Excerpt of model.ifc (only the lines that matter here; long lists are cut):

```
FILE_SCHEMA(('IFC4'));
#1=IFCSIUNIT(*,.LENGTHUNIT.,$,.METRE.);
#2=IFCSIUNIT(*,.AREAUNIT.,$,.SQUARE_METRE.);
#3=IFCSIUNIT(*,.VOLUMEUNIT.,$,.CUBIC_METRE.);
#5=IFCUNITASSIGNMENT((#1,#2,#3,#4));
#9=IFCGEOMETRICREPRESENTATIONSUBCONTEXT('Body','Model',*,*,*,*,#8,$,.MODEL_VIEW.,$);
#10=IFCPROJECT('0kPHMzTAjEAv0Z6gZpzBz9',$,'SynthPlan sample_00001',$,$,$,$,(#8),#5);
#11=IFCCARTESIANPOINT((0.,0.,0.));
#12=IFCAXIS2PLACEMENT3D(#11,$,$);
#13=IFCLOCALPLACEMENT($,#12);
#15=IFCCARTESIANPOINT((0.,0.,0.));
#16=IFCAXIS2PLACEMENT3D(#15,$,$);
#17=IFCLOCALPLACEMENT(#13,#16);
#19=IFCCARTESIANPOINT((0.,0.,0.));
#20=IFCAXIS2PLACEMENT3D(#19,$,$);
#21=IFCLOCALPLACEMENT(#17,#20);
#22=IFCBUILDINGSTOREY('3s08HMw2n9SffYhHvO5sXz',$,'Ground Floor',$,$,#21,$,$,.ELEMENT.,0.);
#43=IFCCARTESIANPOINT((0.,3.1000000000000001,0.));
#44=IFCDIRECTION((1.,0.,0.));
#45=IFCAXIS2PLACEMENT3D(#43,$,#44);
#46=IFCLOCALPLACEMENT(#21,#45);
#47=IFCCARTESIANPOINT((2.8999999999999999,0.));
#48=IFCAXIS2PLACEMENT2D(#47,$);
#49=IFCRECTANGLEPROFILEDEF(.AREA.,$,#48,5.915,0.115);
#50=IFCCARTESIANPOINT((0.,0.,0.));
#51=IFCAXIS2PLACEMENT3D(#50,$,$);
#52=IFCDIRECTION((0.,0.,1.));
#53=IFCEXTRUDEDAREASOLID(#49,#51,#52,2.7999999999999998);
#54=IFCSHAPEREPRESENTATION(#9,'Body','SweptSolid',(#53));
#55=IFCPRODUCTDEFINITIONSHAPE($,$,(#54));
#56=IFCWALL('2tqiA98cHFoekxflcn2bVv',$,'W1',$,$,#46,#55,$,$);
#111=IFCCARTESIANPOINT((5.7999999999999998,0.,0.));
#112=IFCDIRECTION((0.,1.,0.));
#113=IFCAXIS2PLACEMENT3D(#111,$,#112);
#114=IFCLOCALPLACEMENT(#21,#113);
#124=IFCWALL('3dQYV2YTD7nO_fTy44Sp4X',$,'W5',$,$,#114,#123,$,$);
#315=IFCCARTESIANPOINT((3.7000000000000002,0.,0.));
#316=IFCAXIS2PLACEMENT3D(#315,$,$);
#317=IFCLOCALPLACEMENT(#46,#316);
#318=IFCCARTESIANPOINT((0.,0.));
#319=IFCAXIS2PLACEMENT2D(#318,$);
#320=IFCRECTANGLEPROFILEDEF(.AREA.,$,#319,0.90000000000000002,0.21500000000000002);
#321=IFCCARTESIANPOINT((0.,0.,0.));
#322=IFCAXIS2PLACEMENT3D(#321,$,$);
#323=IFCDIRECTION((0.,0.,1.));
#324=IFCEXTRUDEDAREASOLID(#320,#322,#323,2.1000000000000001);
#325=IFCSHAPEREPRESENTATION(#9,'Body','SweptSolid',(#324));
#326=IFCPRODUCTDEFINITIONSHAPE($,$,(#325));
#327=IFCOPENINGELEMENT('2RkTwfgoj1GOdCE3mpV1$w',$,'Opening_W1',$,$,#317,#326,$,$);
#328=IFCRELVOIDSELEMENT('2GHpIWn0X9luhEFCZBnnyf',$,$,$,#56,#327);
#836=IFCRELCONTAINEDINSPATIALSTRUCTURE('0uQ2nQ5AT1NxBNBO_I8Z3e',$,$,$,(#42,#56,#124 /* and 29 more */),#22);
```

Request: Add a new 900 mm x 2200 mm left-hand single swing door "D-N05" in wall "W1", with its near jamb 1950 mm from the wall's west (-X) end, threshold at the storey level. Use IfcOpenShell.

```python
import numpy as np
import ifcopenshell
import ifcopenshell.api.feature
import ifcopenshell.api.geometry
import ifcopenshell.api.root
import ifcopenshell.api.spatial
import ifcopenshell.geom
import ifcopenshell.util.element
import ifcopenshell.util.placement
import ifcopenshell.util.representation
import ifcopenshell.util.shape
import ifcopenshell.util.unit

model = ifcopenshell.open("model.ifc")
unit_scale = ifcopenshell.util.unit.calculate_unit_scale(model)
settings = ifcopenshell.geom.settings()


def volume(element):
    """Net volume in cubic metres, openings subtracted."""
    shape = ifcopenshell.geom.create_shape(settings, element)
    return ifcopenshell.util.shape.get_volume(shape.geometry)


wall = model.by_guid("2tqiA98cHFoekxflcn2bVv")
storey = ifcopenshell.util.element.get_container(wall, ifc_class="IfcBuildingStorey")
context = ifcopenshell.util.representation.get_context(model, "Model", "Body", "MODEL_VIEW")
before = volume(wall)

width, height, from_end, sill = 0.9, 2.2, 1.95, 0.0  # metres

# The wall runs along its own X axis, and the end named is its -X end.
wall_shape = ifcopenshell.geom.create_shape(settings, wall)
x, y, z = ifcopenshell.util.shape.get_vertices(wall_shape.geometry).T
start = x.min() + from_end
face, thickness = float(y.min()), float(y.max() - y.min())
wall_matrix = ifcopenshell.util.placement.get_local_placement(wall.ObjectPlacement)
level = ifcopenshell.util.placement.get_local_placement(storey.ObjectPlacement)[2, 3]


def in_wall(x, y):
    """Placement at x, y metres in the wall's axes, at sill height."""
    matrix = wall_matrix.copy()
    matrix[:, 3] = wall_matrix @ np.array([x / unit_scale, y / unit_scale, 0.0, 1.0])
    matrix[2, 3] = level + sill / unit_scale
    return matrix


# Opening: a box that overshoots both wall faces by 50 mm.
opening = ifcopenshell.api.root.create_entity(model, ifc_class="IfcOpeningElement", predefined_type="OPENING")
box = ifcopenshell.api.geometry.add_wall_representation(
    model, context=context, length=width, height=height, thickness=thickness + 0.1
)
ifcopenshell.api.geometry.assign_representation(model, product=opening, representation=box)
ifcopenshell.api.geometry.edit_object_placement(model, product=opening, matrix=in_wall(start, face - 0.05), is_si=False)
ifcopenshell.api.feature.add_feature(model, feature=opening, element=wall)

door = ifcopenshell.api.root.create_entity(model, ifc_class="IfcDoor", name="D-N05", predefined_type="DOOR")
door.OverallWidth, door.OverallHeight = width / unit_scale, height / unit_scale
door.OperationType = "SINGLE_SWING_LEFT"
body = ifcopenshell.api.geometry.add_door_representation(
    model,
    context=context,
    overall_width=door.OverallWidth,
    overall_height=door.OverallHeight,
    operation_type="SINGLE_SWING_LEFT",
    lining_properties={"LiningDepth": thickness / unit_scale, "ThresholdDepth": thickness / unit_scale},
)
ifcopenshell.api.geometry.assign_representation(model, product=door, representation=body)
ifcopenshell.api.spatial.assign_container(model, products=[door], relating_structure=storey)
ifcopenshell.api.feature.add_filling(model, opening=opening, element=door)

# The lining spans the wall, so the door starts at the wall face.
ifcopenshell.api.geometry.edit_object_placement(model, product=door, matrix=in_wall(start, face), is_si=False)

after = volume(wall)

print(f"wall volume {before:.3f} -> {after:.3f} m3")

model.write("model_rev.ifc")
```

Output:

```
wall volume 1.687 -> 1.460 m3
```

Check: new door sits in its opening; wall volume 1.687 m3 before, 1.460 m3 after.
